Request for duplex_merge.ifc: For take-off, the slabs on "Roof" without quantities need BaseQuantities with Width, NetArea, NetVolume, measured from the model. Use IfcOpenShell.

First a look at what the model holds.

```python
import ifcopenshell
import ifcopenshell.util.element
import ifcopenshell.util.unit

model = ifcopenshell.open("duplex_merge.ifc")
print(model.schema)
for unit_type in ("LENGTHUNIT", "AREAUNIT", "VOLUMEUNIT"):
    print(unit_type, ifcopenshell.util.unit.calculate_unit_scale(model, unit_type))
storey = next(s for s in model.by_type("IfcBuildingStorey") if s.Name == "Roof")
slabs = [e for e in ifcopenshell.util.element.get_decomposition(storey) if e.is_a("IfcSlab")]
for e in sorted(slabs, key=lambda e: e.id()):
    print(e.id(), e.is_a(), e.Name, list(ifcopenshell.util.element.get_psets(e, qtos_only=True)), sep=" | ")
```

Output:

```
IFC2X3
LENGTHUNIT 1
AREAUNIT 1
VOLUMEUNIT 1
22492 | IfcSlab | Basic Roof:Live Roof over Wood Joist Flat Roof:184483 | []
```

```python
import ifcopenshell
import ifcopenshell.api.pset
import ifcopenshell.geom
import ifcopenshell.util.element
import ifcopenshell.util.shape
import ifcopenshell.util.unit

model = ifcopenshell.open("duplex_merge.ifc")
unit_scale = ifcopenshell.util.unit.calculate_unit_scale(model)
area_scale = ifcopenshell.util.unit.calculate_unit_scale(model, "AREAUNIT")
volume_scale = ifcopenshell.util.unit.calculate_unit_scale(model, "VOLUMEUNIT")
settings = ifcopenshell.geom.settings()

storey = next(s for s in model.by_type("IfcBuildingStorey") if s.Name == "Roof")
slabs = [e for e in ifcopenshell.util.element.get_decomposition(storey) if e.is_a("IfcSlab")]

for e in sorted(slabs, key=lambda e: e.id()):
    if ifcopenshell.util.element.get_psets(e, qtos_only=True, should_inherit=False):
        continue
    # Geometry comes back in metres, in the element's own axes.
    shape = ifcopenshell.geom.create_shape(settings, e)
    values = {
        "Width": ifcopenshell.util.shape.get_z(shape.geometry) / unit_scale,
        "NetArea": ifcopenshell.util.shape.get_footprint_area(shape.geometry) / area_scale,
        "NetVolume": ifcopenshell.util.shape.get_volume(shape.geometry) / volume_scale,
    }
    qto = ifcopenshell.api.pset.add_qto(model, product=e, name="BaseQuantities")
    ifcopenshell.api.pset.edit_qto(model, qto=qto, properties=values)
    print(e.id(), {k: round(v, 3) for k, v in values.items()})

model.write("duplex_merge_edited.ifc")
```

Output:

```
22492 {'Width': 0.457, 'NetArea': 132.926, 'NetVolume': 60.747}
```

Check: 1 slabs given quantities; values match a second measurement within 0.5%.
